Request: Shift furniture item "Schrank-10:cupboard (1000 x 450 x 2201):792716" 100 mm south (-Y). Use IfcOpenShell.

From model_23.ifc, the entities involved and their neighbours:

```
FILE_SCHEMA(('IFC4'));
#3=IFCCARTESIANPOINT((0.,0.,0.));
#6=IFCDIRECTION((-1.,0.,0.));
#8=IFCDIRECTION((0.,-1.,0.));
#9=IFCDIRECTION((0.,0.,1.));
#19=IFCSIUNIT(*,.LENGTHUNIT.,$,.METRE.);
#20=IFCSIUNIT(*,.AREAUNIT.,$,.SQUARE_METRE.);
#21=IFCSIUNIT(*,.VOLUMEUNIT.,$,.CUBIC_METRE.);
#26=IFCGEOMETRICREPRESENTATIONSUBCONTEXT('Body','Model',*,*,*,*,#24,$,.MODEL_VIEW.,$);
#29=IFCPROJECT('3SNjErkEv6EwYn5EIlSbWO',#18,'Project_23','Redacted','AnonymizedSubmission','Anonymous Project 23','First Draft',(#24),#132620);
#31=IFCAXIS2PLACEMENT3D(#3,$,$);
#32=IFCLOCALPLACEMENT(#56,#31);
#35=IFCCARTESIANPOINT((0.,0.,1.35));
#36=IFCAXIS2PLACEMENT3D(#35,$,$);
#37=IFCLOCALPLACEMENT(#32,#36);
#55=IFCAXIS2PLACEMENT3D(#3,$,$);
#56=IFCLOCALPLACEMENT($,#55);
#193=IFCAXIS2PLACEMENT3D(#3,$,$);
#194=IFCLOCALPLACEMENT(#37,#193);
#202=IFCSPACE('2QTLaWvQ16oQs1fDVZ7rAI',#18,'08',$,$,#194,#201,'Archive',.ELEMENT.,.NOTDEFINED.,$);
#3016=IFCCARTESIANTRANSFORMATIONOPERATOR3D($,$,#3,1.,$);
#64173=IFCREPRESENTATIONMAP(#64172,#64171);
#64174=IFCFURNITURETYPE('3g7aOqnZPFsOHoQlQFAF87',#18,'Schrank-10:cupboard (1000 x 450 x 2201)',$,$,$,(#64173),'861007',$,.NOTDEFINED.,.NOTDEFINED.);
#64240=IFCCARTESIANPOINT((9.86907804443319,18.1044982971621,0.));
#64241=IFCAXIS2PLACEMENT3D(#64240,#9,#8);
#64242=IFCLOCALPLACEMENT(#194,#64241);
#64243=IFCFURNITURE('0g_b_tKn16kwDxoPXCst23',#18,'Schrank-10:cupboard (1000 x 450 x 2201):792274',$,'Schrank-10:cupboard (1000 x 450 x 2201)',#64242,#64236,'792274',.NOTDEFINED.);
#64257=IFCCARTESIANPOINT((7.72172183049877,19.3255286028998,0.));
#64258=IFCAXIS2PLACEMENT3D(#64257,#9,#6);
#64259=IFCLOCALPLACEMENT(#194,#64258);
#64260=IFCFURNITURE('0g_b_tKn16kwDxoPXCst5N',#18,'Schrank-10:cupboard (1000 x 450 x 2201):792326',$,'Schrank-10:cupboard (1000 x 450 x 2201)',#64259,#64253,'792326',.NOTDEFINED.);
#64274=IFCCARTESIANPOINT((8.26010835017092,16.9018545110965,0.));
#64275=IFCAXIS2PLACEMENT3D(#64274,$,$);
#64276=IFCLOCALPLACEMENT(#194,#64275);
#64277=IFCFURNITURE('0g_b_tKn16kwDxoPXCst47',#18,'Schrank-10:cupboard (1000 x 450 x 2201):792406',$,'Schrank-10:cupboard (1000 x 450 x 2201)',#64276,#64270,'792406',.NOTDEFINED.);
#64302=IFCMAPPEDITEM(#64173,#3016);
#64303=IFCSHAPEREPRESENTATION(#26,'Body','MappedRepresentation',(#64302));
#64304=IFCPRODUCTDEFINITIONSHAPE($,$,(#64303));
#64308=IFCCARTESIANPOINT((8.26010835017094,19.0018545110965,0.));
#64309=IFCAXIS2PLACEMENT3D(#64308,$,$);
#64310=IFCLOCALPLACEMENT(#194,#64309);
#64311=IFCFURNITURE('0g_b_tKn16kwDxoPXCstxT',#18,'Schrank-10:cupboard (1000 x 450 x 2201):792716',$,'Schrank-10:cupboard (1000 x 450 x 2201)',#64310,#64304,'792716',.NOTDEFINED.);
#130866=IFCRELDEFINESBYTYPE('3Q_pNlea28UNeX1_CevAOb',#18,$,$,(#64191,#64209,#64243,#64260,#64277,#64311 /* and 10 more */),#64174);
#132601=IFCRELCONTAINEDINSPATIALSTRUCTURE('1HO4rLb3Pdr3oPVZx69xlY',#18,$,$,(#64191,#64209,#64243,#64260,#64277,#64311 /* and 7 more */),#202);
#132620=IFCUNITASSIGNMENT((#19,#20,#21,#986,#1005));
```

```python
import ifcopenshell
import ifcopenshell.api.geometry
import ifcopenshell.util.placement

model = ifcopenshell.open("model_23.ifc")

item = model.by_guid("0g_b_tKn16kwDxoPXCstxT")
matrix = ifcopenshell.util.placement.get_local_placement(item.ObjectPlacement)
matrix[1, 3] -= 0.1
ifcopenshell.api.geometry.edit_object_placement(model, product=item, matrix=matrix, is_si=False)

print(ifcopenshell.util.placement.get_local_placement(item.ObjectPlacement).round(3) + 0.0)

model.write("model_23_updated.ifc")
```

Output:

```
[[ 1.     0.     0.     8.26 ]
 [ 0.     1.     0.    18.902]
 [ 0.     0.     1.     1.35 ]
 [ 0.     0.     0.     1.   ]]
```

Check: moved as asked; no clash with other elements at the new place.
